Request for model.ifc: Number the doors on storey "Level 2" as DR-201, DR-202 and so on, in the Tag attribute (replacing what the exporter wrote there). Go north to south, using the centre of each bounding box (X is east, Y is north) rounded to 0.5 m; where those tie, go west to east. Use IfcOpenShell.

First a look at what the model holds.

```python
import ifcopenshell
import ifcopenshell.util.element
import ifcopenshell.util.placement

model = ifcopenshell.open("model.ifc")
print(model.schema)
storey = next(s for s in model.by_type("IfcBuildingStorey") if s.Name == "Level 2")
doors = [e for e in ifcopenshell.util.element.get_decomposition(storey) if e.is_a("IfcDoor")]
for e in sorted(doors, key=lambda e: e.id()):
    origin = ifcopenshell.util.placement.get_local_placement(e.ObjectPlacement)[:3, 3]
    print(e.id(), e.Tag, e.Name, origin.round(2) + 0.0, sep=" | ")
```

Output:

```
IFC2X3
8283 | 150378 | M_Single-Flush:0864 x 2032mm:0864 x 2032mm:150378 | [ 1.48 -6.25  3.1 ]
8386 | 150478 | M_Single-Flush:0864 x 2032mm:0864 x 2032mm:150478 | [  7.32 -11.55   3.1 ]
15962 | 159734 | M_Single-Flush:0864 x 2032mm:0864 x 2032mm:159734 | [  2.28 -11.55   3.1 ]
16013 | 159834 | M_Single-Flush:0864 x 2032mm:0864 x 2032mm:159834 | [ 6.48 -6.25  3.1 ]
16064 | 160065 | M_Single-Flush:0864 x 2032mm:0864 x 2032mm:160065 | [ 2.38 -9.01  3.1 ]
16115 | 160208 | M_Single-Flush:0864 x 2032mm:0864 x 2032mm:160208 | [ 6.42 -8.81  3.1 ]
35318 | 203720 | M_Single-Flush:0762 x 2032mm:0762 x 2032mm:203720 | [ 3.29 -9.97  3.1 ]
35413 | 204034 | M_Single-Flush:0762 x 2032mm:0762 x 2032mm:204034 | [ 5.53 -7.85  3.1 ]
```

```python
import ifcopenshell
import ifcopenshell.geom
import ifcopenshell.util.element
import ifcopenshell.util.shape

model = ifcopenshell.open("model.ifc")
settings = ifcopenshell.geom.settings()
settings.set("use-world-coords", True)


def centre(element):
    shape = ifcopenshell.geom.create_shape(settings, element)
    return ifcopenshell.util.shape.get_bbox_centroid(shape.geometry)


storey = next(s for s in model.by_type("IfcBuildingStorey") if s.Name == "Level 2")
doors = [e for e in ifcopenshell.util.element.get_decomposition(storey) if e.is_a("IfcDoor")]

# Insertion points can sit at a corner or the storey origin, so sort by the geometry (in metres).
centres = {e: centre(e) for e in doors}
doors.sort(key=lambda e: (-round(centres[e][1] / 0.5), centres[e][0]))

for i, e in enumerate(doors, start=1):
    number = f"DR-2{i:02d}"
    e.Tag = number
    print(e.id(), number)

model.write("model_updated.ifc")
```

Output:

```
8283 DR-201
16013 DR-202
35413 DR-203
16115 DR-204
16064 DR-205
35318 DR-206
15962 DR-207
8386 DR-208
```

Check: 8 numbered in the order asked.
